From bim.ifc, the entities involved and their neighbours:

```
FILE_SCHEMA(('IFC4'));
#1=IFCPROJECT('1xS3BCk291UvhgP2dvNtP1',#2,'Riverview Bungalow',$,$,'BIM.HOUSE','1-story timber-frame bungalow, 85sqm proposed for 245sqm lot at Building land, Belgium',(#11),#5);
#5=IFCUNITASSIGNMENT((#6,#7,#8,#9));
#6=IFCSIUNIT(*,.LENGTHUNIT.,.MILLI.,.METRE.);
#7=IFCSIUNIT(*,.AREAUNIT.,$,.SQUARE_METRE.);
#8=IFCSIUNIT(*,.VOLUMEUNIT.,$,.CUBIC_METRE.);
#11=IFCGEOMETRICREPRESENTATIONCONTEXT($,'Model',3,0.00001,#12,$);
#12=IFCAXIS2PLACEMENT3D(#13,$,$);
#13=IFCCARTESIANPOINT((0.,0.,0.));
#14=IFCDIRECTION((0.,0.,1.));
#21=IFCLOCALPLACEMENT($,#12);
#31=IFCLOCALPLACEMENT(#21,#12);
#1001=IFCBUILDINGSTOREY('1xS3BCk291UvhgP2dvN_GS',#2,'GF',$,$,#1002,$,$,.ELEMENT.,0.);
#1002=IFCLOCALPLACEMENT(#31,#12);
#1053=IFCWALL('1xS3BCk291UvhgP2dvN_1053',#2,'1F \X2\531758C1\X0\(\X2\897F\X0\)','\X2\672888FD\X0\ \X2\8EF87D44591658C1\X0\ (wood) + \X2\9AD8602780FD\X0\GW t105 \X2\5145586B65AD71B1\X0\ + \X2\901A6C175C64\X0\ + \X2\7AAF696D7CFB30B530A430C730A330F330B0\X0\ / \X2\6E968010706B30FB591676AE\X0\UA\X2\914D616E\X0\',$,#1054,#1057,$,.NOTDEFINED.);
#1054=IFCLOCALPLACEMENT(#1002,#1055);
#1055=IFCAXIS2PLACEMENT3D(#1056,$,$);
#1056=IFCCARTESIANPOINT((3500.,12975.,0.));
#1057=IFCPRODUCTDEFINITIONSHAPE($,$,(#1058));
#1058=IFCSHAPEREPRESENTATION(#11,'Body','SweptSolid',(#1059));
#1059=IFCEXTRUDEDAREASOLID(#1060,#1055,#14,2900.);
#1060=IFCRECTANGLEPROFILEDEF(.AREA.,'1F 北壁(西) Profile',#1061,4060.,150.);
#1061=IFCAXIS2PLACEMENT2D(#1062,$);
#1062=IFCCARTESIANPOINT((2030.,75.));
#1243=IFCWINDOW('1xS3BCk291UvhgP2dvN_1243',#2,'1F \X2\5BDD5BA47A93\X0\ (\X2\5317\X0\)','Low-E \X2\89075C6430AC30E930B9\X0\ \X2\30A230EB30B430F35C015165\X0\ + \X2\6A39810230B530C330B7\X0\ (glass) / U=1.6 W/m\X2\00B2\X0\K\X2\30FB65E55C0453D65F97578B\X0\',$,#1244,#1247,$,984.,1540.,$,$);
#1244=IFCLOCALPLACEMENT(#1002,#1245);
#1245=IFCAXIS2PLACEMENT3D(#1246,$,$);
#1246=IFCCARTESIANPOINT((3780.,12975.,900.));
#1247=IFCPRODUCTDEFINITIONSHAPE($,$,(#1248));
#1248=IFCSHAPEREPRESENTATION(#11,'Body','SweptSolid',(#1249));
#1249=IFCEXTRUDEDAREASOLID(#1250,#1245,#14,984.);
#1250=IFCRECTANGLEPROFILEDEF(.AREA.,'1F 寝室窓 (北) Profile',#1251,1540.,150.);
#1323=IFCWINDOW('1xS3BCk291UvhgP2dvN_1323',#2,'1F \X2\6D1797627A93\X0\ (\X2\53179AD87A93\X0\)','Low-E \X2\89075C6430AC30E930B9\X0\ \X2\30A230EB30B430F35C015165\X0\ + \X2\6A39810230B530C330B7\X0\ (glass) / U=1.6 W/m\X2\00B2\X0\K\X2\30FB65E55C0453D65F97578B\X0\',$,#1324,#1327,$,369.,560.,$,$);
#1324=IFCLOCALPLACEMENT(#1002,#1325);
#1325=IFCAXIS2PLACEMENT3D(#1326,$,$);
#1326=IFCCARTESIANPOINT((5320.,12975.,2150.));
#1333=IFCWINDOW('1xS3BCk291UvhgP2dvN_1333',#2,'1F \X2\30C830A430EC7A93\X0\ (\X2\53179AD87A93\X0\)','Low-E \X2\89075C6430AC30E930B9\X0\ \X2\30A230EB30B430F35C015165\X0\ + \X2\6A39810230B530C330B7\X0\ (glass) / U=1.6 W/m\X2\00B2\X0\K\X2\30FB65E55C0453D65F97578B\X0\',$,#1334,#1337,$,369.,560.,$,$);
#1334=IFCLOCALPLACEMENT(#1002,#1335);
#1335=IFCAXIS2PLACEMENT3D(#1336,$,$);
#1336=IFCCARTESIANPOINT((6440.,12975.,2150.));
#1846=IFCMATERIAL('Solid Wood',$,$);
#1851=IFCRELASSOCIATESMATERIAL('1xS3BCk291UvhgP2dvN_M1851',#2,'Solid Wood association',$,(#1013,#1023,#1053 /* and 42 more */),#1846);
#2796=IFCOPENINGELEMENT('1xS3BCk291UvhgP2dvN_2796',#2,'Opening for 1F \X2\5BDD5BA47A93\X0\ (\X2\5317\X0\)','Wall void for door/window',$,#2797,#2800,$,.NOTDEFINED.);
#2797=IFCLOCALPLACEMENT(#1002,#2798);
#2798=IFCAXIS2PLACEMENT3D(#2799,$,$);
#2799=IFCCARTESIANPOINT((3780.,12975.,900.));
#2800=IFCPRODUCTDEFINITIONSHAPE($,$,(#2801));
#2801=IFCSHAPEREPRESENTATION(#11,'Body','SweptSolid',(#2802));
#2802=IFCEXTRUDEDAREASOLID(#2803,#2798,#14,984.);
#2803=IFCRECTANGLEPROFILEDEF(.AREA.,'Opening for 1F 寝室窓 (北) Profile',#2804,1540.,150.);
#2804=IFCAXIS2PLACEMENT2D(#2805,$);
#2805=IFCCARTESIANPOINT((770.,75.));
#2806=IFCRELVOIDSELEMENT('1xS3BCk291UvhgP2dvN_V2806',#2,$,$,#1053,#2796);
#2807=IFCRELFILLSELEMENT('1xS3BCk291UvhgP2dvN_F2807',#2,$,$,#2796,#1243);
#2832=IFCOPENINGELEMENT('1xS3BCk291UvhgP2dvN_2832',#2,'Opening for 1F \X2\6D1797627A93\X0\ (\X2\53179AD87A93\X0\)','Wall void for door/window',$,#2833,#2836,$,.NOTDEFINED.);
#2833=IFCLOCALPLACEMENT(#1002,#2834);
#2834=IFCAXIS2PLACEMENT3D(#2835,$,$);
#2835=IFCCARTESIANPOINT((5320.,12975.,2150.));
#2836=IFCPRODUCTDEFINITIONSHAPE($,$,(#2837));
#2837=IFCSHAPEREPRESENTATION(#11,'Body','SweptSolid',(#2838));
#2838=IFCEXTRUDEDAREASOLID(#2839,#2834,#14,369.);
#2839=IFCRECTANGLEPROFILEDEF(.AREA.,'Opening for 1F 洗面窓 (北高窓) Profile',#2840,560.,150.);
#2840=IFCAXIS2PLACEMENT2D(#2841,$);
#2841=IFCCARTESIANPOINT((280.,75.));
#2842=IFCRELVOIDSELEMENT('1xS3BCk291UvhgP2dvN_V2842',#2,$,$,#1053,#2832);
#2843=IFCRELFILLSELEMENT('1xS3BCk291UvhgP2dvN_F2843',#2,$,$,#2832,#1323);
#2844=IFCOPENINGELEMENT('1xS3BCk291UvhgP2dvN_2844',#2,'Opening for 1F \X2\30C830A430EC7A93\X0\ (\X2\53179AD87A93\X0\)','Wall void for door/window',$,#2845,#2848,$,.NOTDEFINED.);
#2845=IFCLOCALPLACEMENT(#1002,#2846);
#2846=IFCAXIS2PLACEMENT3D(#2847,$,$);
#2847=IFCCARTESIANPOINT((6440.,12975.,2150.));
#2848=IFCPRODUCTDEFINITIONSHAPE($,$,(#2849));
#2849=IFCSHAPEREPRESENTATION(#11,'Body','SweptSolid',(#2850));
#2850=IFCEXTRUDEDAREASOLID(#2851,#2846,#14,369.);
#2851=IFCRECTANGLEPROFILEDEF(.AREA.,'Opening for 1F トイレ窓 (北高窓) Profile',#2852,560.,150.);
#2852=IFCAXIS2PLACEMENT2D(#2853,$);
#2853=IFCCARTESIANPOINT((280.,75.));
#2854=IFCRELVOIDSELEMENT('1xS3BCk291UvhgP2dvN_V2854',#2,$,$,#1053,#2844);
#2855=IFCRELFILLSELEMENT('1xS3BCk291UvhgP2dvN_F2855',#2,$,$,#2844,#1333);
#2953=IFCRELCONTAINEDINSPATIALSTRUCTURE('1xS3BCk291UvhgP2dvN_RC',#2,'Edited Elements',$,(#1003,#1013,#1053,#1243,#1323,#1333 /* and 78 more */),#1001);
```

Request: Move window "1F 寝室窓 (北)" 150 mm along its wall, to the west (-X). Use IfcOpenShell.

```python
import ifcopenshell
import ifcopenshell.api.geometry
import ifcopenshell.util.placement
import ifcopenshell.util.unit

model = ifcopenshell.open("bim.ifc")
unit_scale = ifcopenshell.util.unit.calculate_unit_scale(model)

window = model.by_guid("1xS3BCk291UvhgP2dvN_1243")
opening = window.FillsVoids[0].RelatingOpeningElement
wall = opening.VoidsElements[0].RelatingBuildingElement

wall_matrix = ifcopenshell.util.placement.get_local_placement(wall.ObjectPlacement)
shift = wall_matrix[:3, 0] * -0.15 / unit_scale
before = ifcopenshell.util.placement.get_local_placement(window.ObjectPlacement)[:3, 3].copy()

# The window is not placed relative to its opening, so move both.
for product in (opening, window):
    matrix = ifcopenshell.util.placement.get_local_placement(product.ObjectPlacement)
    matrix[:3, 3] += shift
    ifcopenshell.api.geometry.edit_object_placement(model, product=product, matrix=matrix, is_si=False)

after = ifcopenshell.util.placement.get_local_placement(window.ObjectPlacement)[:3, 3]
print("window moved by", (after - before).round(3) + 0.0)

model.write("bim_v2.ifc")
```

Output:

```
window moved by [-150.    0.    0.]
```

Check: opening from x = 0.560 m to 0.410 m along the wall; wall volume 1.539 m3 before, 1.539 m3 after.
